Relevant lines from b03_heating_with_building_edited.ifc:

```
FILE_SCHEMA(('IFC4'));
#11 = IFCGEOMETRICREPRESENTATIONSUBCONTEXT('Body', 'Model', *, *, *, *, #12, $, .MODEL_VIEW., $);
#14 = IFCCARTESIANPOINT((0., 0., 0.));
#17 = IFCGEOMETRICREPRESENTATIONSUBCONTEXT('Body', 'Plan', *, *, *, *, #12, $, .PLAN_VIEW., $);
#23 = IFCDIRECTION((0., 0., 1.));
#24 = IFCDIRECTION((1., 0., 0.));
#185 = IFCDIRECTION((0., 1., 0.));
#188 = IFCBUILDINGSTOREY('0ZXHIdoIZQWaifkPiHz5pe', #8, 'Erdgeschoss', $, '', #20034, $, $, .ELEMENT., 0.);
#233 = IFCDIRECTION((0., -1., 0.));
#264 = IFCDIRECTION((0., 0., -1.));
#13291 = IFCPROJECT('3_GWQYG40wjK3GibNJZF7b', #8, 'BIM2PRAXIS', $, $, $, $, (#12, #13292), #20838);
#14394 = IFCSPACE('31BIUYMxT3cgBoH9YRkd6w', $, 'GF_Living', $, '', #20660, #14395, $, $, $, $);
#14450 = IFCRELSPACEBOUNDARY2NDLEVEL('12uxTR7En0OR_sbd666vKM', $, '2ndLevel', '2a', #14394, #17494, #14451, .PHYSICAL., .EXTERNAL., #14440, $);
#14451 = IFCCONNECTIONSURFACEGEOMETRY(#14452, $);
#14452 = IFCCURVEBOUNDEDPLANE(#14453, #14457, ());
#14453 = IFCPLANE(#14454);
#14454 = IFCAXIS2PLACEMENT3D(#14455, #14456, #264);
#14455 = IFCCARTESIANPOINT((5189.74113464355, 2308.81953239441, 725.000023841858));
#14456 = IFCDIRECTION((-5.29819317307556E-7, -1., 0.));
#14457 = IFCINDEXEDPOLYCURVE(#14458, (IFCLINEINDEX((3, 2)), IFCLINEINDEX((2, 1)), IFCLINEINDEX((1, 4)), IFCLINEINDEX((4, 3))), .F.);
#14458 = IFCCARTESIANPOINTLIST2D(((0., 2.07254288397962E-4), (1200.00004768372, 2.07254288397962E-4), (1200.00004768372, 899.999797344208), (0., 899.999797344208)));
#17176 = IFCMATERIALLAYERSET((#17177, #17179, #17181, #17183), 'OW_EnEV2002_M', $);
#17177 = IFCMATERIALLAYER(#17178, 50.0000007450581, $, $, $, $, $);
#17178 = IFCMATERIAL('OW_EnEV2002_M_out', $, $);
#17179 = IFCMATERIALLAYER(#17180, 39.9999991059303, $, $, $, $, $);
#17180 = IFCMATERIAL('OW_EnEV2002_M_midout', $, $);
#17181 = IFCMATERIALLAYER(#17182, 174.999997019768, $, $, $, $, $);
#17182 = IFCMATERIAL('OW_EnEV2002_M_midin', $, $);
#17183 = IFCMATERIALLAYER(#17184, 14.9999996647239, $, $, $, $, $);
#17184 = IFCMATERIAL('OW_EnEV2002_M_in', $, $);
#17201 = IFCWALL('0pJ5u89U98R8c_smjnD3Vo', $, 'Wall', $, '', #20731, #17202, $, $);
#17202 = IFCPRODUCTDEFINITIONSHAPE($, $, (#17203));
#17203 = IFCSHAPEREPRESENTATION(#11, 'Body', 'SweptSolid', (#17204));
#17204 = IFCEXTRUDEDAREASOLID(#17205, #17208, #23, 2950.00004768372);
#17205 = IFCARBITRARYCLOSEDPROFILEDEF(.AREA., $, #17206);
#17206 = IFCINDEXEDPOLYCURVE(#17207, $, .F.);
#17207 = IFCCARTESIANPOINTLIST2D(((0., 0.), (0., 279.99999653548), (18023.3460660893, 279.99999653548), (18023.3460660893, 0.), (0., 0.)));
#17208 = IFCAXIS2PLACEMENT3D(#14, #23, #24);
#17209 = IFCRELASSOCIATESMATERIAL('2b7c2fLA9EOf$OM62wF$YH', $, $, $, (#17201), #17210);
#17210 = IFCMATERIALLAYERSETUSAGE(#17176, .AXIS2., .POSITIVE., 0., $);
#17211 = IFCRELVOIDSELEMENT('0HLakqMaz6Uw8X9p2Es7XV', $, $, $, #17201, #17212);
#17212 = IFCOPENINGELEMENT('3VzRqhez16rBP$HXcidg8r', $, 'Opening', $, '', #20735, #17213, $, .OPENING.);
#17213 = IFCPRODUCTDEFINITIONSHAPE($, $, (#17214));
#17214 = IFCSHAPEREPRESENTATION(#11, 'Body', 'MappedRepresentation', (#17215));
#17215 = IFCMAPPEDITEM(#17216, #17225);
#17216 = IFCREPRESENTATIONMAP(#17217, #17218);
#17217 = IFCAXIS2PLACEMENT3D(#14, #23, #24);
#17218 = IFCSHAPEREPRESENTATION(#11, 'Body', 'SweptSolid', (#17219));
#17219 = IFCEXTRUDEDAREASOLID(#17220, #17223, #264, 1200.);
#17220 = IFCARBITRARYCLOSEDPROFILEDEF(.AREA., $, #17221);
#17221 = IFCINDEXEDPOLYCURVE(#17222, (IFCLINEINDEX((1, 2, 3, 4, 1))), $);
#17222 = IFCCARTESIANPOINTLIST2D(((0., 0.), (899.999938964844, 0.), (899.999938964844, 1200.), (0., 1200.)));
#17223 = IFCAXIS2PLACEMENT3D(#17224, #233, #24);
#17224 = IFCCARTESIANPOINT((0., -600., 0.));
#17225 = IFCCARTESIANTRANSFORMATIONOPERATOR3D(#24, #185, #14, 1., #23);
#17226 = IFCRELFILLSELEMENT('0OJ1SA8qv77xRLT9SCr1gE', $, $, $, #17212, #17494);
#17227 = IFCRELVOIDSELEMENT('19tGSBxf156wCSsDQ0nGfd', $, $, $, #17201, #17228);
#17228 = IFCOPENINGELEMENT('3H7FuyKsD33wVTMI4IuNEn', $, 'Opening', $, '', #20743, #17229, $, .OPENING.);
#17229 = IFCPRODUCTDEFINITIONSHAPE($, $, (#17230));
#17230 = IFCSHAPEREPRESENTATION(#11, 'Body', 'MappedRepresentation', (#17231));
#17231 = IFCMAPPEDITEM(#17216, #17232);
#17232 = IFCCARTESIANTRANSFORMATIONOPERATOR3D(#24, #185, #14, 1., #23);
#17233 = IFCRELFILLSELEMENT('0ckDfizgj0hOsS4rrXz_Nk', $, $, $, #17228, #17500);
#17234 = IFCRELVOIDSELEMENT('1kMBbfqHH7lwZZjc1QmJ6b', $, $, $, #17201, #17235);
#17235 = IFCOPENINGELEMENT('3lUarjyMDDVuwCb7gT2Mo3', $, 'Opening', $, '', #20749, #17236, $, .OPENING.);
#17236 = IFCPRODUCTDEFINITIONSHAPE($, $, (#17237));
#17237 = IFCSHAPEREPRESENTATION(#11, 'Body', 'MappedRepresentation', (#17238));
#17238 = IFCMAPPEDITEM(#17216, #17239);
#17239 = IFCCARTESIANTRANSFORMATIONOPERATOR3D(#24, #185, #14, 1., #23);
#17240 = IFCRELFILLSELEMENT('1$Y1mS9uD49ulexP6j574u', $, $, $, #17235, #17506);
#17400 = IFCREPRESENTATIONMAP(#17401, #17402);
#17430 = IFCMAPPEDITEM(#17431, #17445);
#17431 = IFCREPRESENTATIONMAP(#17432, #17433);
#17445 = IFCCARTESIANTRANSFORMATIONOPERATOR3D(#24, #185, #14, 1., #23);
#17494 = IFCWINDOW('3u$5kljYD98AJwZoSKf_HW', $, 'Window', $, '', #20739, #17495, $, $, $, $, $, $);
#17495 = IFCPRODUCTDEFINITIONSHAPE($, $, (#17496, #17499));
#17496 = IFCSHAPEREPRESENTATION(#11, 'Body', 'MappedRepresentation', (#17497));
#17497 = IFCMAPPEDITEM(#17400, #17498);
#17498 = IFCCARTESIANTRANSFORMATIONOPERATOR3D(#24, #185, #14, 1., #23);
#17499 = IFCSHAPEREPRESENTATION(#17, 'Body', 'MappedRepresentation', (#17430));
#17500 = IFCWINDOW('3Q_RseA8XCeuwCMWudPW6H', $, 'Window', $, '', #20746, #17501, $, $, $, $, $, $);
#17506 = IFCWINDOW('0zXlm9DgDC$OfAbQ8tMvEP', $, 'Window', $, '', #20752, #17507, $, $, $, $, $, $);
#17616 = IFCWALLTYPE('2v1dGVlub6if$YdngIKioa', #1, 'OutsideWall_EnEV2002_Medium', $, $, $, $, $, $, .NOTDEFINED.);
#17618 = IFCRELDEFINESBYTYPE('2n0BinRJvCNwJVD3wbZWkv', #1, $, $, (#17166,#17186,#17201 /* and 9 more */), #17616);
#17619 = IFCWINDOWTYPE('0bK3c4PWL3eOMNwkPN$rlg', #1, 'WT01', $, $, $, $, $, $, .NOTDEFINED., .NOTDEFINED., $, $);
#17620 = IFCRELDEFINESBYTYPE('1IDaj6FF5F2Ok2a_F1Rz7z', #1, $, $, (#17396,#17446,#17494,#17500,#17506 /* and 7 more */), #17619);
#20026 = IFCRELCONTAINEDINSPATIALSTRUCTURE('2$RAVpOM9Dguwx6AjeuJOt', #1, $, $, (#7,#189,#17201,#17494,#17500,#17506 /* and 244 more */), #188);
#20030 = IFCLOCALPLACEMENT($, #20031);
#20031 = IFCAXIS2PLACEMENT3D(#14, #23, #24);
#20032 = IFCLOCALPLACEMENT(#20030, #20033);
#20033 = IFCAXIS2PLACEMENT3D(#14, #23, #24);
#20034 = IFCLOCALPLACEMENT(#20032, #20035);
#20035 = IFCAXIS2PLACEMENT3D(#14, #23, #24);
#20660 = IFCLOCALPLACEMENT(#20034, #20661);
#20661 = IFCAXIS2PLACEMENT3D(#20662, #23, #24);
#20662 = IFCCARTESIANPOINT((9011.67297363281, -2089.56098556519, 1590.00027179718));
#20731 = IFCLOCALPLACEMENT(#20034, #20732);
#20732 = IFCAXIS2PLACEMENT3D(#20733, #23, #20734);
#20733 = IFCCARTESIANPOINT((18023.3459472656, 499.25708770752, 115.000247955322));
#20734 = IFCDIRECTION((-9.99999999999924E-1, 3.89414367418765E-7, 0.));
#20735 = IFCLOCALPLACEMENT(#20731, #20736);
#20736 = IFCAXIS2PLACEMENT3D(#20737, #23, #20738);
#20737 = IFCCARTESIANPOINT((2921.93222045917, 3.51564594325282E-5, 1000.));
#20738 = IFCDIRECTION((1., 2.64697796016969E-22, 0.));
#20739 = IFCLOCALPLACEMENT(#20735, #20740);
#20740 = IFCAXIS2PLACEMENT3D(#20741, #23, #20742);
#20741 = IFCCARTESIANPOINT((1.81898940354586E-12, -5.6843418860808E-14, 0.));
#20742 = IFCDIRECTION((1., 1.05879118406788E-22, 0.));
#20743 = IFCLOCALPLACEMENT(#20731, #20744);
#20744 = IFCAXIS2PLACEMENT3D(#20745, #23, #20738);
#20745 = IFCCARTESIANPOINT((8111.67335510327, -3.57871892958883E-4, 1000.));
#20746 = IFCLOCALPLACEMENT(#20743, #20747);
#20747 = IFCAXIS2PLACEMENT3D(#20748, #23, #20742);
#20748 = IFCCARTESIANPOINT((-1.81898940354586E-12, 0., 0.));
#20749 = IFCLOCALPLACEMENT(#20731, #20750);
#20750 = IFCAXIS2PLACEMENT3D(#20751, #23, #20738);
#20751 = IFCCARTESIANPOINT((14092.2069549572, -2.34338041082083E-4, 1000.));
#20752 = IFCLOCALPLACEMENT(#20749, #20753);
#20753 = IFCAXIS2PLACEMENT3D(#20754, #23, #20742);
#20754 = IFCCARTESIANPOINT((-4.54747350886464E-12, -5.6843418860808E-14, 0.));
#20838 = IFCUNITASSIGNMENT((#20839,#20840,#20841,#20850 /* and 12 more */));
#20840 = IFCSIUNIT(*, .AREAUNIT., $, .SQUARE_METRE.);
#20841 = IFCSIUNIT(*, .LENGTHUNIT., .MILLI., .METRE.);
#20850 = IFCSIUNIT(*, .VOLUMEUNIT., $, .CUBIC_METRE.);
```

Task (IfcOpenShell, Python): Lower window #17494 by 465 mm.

```python
import numpy as np
import ifcopenshell
import ifcopenshell.api.geometry
import ifcopenshell.util.placement
import ifcopenshell.util.unit

model = ifcopenshell.open("b03_heating_with_building_edited.ifc")
unit_scale = ifcopenshell.util.unit.calculate_unit_scale(model)

window = model.by_guid("3u$5kljYD98AJwZoSKf_HW")
opening = window.FillsVoids[0].RelatingOpeningElement
dz = -0.465 / unit_scale

shift = np.array([0.0, 0.0, dz])
# The window is placed relative to its opening, so it follows when the opening moves.
matrix = ifcopenshell.util.placement.get_local_placement(opening.ObjectPlacement)
matrix[:3, 3] += shift
ifcopenshell.api.geometry.edit_object_placement(
    model, product=opening, matrix=matrix, is_si=False, should_transform_children=True
)

# Space boundary surfaces are stored in each space's coordinates; move them too.
for rel in window.ProvidesBoundaries:
    if not rel.ConnectionGeometry:
        continue
    surface = rel.ConnectionGeometry.SurfaceOnRelatingElement.BasisSurface
    space_matrix = ifcopenshell.util.placement.get_local_placement(rel.RelatingSpace.ObjectPlacement)
    point = np.array(surface.Position.Location.Coordinates) + space_matrix[:3, :3].T @ shift
    surface.Position = model.createIfcAxis2Placement3D(
        model.createIfcCartesianPoint(point.tolist()), surface.Position.Axis, surface.Position.RefDirection
    )

print(f"moved by {dz * unit_scale:+.3f} m")

model.write("b03_heating_with_building_edited-out.ifc")
```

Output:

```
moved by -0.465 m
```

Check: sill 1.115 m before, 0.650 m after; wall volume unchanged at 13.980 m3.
